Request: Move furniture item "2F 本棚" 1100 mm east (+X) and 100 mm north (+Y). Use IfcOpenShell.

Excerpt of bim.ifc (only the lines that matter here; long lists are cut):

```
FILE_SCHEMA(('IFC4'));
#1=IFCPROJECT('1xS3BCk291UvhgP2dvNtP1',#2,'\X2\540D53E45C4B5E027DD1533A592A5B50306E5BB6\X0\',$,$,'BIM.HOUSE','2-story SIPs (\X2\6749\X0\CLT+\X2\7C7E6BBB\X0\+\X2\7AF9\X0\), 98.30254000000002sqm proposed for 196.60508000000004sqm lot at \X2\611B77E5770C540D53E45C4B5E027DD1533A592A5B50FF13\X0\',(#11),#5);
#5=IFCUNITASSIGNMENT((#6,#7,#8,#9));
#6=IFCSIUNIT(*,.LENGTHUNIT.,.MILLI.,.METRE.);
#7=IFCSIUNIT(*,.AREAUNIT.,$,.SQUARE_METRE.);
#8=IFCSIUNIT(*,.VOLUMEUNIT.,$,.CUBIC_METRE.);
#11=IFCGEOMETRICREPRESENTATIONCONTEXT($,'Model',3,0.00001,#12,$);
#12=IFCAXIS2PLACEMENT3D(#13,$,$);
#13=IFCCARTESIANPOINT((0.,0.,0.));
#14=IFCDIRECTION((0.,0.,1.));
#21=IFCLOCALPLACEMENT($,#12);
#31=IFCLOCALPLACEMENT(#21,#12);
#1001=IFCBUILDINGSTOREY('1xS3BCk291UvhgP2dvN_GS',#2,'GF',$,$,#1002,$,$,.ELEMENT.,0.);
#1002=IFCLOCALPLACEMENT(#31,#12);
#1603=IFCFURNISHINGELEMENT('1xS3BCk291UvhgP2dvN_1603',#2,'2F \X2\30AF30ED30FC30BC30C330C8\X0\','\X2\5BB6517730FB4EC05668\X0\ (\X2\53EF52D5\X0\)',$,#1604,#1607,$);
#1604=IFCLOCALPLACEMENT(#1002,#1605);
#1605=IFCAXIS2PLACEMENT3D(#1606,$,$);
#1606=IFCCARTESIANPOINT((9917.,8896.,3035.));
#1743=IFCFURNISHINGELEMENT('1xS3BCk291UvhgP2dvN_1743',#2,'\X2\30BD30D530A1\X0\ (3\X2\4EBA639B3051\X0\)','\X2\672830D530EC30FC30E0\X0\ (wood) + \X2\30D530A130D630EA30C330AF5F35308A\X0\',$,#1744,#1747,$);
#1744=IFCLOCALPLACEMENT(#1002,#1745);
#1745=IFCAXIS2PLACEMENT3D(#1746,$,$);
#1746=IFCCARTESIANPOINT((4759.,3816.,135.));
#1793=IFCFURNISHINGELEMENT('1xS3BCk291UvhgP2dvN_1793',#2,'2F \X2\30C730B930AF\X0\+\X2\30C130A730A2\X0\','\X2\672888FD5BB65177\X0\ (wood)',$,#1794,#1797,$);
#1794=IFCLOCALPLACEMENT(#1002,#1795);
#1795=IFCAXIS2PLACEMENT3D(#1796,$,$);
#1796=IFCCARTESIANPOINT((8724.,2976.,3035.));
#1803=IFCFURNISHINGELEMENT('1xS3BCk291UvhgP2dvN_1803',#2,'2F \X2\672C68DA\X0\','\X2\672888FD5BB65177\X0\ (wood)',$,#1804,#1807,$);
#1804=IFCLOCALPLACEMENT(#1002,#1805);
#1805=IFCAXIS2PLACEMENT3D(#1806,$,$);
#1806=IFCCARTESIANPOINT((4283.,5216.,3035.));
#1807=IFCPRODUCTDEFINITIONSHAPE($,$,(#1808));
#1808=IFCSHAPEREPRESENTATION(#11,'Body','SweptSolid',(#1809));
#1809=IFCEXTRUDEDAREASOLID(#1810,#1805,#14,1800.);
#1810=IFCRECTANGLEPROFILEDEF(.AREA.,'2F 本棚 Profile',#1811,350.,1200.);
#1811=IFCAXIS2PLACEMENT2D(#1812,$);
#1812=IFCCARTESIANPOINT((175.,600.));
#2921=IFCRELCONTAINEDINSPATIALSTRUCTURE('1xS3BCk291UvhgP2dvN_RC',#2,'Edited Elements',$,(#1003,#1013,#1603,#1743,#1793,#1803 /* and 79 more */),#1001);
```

```python
import ifcopenshell
import ifcopenshell.api.geometry
import ifcopenshell.util.placement
import ifcopenshell.util.unit

model = ifcopenshell.open("bim.ifc")
unit_scale = ifcopenshell.util.unit.calculate_unit_scale(model)

item = model.by_guid("1xS3BCk291UvhgP2dvN_1803")
matrix = ifcopenshell.util.placement.get_local_placement(item.ObjectPlacement)
matrix[0, 3] += 1.1 / unit_scale
matrix[1, 3] += 0.1 / unit_scale
ifcopenshell.api.geometry.edit_object_placement(model, product=item, matrix=matrix, is_si=False)

print(ifcopenshell.util.placement.get_local_placement(item.ObjectPlacement).round(3) + 0.0)

model.write("bim_edited.ifc")
```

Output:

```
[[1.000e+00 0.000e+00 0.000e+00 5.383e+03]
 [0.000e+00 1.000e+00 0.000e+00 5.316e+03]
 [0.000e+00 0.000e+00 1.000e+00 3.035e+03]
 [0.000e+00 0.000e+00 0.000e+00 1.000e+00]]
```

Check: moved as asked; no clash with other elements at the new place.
